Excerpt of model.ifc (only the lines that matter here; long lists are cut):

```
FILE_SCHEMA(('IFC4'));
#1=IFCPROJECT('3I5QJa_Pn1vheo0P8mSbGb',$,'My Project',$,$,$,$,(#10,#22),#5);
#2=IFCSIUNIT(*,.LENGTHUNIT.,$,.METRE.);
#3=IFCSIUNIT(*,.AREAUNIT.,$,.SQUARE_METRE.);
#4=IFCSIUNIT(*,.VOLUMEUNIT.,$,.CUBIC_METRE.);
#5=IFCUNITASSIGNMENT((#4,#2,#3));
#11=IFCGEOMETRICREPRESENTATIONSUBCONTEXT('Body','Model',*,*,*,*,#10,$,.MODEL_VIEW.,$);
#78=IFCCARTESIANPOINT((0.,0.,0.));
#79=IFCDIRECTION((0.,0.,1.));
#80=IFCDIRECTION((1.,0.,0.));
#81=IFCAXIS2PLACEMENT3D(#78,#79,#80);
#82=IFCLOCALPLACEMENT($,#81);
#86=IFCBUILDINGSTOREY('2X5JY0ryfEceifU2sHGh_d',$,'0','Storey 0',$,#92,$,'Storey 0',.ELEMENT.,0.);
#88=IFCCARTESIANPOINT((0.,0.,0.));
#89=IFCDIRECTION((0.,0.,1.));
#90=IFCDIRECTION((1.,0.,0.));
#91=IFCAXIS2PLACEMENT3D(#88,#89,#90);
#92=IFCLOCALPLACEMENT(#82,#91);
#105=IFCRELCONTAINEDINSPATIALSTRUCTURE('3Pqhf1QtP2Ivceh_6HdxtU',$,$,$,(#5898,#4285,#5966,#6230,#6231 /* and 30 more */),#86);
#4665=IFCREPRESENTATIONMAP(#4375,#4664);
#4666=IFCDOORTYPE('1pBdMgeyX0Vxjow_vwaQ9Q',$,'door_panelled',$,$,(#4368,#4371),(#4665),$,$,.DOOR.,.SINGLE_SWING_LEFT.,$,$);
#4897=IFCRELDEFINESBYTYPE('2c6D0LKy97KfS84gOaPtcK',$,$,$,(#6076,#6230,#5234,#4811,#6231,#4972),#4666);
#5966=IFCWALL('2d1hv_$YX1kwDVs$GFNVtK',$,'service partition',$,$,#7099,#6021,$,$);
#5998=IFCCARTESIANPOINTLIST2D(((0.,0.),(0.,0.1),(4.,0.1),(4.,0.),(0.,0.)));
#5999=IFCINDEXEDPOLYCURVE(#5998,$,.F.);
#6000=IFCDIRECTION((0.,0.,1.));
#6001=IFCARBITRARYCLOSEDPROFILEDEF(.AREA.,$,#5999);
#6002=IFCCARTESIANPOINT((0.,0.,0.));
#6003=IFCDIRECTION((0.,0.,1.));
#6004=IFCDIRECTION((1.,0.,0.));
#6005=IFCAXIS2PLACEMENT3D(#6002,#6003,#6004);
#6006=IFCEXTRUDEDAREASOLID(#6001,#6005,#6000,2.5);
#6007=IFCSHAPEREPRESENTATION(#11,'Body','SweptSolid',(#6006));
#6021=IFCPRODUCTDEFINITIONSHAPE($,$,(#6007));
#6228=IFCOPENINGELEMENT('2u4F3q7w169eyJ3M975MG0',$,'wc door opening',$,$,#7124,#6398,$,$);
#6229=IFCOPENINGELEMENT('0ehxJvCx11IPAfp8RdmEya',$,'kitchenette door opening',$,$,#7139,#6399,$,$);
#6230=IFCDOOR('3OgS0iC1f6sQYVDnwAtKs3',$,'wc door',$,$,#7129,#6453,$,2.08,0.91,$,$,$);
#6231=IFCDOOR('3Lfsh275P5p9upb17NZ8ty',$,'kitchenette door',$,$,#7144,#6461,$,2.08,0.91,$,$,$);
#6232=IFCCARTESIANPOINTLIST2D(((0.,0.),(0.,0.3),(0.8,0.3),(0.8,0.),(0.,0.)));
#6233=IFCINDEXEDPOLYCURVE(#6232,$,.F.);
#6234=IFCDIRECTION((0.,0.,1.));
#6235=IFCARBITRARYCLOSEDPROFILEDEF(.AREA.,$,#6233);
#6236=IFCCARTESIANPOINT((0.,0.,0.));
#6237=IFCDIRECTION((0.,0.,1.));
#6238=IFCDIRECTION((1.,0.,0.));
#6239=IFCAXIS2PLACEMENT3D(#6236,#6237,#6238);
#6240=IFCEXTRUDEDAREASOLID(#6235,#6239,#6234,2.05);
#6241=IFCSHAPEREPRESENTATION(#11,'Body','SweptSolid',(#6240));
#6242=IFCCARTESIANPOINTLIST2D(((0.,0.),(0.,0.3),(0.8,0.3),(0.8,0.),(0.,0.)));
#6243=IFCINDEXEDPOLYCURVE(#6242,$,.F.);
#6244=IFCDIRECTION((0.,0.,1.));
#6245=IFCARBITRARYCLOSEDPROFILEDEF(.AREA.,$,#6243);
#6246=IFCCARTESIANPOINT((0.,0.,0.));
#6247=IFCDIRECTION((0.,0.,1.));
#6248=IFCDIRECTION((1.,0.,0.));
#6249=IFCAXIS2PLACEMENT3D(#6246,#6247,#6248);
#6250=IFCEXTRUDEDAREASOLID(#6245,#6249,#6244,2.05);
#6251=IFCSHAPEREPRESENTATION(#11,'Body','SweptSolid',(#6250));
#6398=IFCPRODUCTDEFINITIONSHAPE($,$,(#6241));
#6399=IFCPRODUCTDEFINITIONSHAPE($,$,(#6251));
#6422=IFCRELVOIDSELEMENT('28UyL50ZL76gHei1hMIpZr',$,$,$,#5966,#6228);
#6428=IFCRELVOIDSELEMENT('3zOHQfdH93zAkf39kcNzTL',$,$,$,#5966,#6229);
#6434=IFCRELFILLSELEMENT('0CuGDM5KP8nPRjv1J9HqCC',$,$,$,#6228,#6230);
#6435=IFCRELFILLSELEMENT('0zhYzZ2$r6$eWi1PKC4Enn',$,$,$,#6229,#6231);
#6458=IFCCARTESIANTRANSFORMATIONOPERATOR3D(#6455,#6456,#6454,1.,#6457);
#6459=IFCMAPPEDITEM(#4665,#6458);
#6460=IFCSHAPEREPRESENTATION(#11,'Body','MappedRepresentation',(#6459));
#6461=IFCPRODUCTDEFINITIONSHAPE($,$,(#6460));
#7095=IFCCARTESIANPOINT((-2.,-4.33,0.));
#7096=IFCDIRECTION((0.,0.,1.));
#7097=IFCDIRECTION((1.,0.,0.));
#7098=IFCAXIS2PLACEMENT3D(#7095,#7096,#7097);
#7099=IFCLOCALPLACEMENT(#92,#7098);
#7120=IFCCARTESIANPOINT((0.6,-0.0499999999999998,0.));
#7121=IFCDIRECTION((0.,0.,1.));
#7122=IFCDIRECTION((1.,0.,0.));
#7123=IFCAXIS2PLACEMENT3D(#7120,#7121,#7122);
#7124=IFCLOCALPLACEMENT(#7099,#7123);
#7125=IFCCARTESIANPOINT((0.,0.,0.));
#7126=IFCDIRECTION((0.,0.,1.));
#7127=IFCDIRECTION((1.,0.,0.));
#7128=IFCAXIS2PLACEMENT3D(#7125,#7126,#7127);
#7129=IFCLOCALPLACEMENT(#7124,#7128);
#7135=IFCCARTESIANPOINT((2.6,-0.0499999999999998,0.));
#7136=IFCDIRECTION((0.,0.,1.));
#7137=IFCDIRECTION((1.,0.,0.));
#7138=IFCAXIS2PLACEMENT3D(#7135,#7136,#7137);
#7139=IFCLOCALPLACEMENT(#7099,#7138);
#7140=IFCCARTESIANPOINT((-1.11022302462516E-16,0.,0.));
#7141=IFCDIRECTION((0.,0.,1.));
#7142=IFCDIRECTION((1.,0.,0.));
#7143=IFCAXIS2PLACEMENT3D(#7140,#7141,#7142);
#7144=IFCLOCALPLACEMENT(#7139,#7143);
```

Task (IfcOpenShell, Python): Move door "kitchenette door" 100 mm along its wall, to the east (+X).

```python
import ifcopenshell
import ifcopenshell.api.geometry
import ifcopenshell.util.placement
import ifcopenshell.util.unit

model = ifcopenshell.open("model.ifc")
unit_scale = ifcopenshell.util.unit.calculate_unit_scale(model)

door = model.by_id(6231)
opening = door.FillsVoids[0].RelatingOpeningElement
wall = opening.VoidsElements[0].RelatingBuildingElement

wall_matrix = ifcopenshell.util.placement.get_local_placement(wall.ObjectPlacement)
shift = wall_matrix[:3, 0] * 0.1 / unit_scale
before = ifcopenshell.util.placement.get_local_placement(door.ObjectPlacement)[:3, 3].copy()

# The door is placed relative to its opening, so it follows when the opening moves.
matrix = ifcopenshell.util.placement.get_local_placement(opening.ObjectPlacement)
matrix[:3, 3] += shift
ifcopenshell.api.geometry.edit_object_placement(
    model, product=opening, matrix=matrix, is_si=False, should_transform_children=True
)

after = ifcopenshell.util.placement.get_local_placement(door.ObjectPlacement)[:3, 3]
print("door moved by", (after - before).round(3) + 0.0)

model.write("model_edited.ifc")
```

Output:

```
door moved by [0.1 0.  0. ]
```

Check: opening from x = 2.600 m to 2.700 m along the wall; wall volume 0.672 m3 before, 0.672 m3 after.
